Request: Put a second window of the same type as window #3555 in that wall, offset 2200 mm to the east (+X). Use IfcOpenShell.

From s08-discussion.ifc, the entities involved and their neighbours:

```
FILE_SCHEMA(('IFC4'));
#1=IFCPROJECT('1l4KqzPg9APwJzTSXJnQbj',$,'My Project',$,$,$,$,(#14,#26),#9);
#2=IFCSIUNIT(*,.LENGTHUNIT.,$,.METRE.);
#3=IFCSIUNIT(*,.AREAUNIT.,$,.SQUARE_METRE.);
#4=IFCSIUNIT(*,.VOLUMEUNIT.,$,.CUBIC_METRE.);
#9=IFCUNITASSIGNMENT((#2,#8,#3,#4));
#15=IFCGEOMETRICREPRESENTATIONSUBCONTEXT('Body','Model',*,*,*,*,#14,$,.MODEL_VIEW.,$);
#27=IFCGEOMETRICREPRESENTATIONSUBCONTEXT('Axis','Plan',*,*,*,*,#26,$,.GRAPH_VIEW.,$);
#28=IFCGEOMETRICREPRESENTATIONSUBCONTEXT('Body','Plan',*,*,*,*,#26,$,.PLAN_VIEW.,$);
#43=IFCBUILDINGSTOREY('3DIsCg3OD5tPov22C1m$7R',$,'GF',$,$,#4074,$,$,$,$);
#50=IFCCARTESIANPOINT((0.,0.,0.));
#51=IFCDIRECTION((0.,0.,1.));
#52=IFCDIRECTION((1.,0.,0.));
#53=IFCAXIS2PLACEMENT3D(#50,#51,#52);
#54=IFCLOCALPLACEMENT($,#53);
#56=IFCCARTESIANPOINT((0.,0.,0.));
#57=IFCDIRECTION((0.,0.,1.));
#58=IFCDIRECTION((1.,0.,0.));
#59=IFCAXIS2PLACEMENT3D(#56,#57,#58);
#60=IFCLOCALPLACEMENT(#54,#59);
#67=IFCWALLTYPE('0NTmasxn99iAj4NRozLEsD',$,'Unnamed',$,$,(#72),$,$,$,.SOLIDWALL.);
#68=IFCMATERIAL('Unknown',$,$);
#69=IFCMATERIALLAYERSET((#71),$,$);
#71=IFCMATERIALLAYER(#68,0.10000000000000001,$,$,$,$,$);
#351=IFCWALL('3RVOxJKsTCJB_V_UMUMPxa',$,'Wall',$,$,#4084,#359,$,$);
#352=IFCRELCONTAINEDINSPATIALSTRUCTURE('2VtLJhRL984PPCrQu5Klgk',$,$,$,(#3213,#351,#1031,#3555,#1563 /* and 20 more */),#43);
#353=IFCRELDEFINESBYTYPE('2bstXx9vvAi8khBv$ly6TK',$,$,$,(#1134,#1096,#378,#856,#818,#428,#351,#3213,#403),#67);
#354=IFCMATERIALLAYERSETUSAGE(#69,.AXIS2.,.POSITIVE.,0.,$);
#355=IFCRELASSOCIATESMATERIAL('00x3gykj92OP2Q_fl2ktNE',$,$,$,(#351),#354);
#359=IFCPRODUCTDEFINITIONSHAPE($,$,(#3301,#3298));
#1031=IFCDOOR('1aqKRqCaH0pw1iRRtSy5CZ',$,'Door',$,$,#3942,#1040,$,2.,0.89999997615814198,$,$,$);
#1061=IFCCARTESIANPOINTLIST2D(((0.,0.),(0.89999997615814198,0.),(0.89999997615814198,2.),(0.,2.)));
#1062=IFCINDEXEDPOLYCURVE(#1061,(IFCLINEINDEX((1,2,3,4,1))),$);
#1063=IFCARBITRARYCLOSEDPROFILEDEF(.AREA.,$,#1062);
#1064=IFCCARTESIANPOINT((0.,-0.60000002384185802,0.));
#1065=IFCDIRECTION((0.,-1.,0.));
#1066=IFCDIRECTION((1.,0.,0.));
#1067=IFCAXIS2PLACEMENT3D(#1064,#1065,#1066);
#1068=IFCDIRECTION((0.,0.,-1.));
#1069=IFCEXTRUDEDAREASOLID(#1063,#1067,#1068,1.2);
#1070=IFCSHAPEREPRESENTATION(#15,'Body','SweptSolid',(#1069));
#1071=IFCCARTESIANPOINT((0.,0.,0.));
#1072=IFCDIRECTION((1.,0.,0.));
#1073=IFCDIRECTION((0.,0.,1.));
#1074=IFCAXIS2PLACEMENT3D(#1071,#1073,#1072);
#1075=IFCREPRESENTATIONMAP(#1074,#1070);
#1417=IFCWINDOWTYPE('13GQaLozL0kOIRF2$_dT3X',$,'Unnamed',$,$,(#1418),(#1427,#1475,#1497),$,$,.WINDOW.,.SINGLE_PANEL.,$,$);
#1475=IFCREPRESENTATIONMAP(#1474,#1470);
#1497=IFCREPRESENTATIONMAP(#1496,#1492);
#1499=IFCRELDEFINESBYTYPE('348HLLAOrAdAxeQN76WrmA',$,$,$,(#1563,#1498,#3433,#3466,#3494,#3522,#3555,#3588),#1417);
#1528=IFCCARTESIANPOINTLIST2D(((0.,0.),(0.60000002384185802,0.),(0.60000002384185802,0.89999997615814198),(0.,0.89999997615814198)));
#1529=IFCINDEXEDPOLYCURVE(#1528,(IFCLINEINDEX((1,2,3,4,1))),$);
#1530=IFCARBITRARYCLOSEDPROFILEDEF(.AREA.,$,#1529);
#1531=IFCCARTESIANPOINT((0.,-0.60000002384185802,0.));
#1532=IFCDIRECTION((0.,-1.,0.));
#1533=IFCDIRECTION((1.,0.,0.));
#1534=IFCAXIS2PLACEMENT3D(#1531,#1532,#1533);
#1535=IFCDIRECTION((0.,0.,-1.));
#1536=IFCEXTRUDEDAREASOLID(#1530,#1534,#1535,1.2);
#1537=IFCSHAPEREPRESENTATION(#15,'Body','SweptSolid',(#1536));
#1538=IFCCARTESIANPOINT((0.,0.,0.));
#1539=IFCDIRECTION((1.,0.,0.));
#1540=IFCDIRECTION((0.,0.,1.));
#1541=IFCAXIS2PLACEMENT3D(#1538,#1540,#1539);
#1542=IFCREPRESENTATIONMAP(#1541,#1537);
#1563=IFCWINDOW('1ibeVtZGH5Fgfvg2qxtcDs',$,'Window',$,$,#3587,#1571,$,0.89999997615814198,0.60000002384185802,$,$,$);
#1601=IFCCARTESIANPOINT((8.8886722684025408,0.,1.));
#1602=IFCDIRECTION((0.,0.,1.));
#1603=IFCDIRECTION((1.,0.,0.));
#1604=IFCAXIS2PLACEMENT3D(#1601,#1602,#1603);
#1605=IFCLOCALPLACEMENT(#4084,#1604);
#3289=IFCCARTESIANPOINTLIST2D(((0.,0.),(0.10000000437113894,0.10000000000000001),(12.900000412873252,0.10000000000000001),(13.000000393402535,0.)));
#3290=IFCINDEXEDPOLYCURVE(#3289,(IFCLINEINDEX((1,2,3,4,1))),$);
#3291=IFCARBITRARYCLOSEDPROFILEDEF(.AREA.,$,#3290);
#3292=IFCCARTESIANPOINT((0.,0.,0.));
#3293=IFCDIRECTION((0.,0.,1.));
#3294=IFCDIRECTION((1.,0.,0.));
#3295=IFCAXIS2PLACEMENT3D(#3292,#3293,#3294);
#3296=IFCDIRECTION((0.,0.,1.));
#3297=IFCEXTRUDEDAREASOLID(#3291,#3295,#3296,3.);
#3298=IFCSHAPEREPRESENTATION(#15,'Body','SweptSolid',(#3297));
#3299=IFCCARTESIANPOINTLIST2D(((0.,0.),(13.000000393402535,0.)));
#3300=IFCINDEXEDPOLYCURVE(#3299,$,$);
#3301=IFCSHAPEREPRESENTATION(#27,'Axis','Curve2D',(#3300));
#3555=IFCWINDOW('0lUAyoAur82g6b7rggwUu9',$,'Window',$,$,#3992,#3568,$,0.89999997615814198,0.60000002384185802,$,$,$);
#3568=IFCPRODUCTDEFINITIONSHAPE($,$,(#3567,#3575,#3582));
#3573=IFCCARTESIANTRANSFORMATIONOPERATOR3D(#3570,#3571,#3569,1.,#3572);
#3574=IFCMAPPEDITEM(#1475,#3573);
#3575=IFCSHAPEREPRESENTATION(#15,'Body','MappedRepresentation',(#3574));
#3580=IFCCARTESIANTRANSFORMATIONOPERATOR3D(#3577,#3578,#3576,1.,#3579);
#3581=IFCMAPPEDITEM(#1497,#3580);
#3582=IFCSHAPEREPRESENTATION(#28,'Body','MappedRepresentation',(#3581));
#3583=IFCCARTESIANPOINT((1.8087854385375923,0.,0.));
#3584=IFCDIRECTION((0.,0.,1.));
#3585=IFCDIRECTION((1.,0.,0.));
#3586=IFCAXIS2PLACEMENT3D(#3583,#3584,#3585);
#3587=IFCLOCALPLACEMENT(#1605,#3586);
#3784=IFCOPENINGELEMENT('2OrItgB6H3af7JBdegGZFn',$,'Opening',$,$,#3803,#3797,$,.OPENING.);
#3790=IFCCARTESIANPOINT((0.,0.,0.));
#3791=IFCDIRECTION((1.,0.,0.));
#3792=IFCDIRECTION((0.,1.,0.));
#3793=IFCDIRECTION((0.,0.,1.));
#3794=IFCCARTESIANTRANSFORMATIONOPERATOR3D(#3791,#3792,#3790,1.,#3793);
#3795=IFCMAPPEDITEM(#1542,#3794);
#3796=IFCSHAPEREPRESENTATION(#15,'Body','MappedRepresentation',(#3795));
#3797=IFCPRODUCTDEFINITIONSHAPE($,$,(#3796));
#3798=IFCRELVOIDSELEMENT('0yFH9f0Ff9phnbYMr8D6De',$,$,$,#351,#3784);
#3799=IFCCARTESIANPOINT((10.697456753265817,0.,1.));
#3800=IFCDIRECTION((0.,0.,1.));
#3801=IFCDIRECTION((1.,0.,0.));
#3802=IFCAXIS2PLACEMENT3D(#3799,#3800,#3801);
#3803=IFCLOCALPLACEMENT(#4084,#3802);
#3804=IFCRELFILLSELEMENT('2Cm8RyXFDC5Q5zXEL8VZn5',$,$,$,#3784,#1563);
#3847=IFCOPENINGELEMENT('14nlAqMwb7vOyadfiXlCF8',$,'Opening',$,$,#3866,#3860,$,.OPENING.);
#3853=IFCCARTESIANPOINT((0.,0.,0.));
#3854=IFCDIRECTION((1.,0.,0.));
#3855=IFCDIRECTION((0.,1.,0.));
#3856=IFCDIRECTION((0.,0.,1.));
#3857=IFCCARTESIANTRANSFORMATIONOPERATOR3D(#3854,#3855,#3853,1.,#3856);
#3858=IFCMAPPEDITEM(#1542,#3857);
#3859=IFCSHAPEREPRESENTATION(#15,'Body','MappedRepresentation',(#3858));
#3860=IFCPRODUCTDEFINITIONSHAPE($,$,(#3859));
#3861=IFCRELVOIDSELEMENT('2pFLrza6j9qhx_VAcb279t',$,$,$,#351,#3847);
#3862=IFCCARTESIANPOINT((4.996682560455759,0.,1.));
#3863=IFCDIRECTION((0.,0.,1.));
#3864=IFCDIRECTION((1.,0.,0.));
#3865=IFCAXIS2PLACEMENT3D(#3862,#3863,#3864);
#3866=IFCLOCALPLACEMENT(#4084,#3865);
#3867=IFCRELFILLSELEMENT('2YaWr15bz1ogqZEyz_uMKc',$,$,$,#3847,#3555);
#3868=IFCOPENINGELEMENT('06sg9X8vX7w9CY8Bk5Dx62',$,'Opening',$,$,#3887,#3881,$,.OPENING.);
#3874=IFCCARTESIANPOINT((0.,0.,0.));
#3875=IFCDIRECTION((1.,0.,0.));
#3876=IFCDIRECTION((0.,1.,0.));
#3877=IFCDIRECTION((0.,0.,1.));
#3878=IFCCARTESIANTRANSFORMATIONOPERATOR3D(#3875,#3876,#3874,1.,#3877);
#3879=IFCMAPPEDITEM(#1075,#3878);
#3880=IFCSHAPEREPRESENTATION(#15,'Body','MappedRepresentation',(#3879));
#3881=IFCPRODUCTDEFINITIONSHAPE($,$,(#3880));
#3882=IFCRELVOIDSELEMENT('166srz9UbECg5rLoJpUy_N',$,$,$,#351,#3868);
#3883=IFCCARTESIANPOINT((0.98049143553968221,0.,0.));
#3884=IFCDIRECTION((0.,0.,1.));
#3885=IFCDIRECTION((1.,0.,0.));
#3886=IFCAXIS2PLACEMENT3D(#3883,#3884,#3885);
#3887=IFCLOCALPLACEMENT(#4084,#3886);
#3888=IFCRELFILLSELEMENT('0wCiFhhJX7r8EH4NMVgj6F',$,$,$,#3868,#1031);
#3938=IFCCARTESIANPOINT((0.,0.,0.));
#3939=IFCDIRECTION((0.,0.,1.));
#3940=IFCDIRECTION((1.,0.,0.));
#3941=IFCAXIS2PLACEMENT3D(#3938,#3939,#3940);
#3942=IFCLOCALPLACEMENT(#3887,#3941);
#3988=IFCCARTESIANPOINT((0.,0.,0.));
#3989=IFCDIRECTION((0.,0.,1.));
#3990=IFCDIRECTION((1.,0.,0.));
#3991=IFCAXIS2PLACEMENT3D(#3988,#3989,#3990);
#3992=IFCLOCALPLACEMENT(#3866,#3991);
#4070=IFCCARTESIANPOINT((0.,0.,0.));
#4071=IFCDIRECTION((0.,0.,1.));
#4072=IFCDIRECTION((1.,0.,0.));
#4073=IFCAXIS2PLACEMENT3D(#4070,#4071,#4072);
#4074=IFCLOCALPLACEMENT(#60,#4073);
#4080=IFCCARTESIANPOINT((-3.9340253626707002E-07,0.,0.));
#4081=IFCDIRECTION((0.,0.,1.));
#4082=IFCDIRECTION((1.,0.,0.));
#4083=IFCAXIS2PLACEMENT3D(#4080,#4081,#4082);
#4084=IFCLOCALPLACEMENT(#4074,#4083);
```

```python
import ifcopenshell
import ifcopenshell.api.feature
import ifcopenshell.api.geometry
import ifcopenshell.api.root
import ifcopenshell.geom
import ifcopenshell.util.element
import ifcopenshell.util.placement
import ifcopenshell.util.shape
import ifcopenshell.util.unit

model = ifcopenshell.open("s08-discussion.ifc")
unit_scale = ifcopenshell.util.unit.calculate_unit_scale(model)
settings = ifcopenshell.geom.settings()


def volume(element):
    """Net volume in cubic metres, openings subtracted."""
    shape = ifcopenshell.geom.create_shape(settings, element)
    return ifcopenshell.util.shape.get_volume(shape.geometry)


window = model.by_guid("0lUAyoAur82g6b7rggwUu9")
opening = window.FillsVoids[0].RelatingOpeningElement
wall = opening.VoidsElements[0].RelatingBuildingElement
before = volume(wall)
shift = ifcopenshell.util.placement.get_local_placement(wall.ObjectPlacement)[:3, 0] * 2.2 / unit_scale

# copy_class copies the void relationship, type, container and properties, but no geometry.
new_opening = ifcopenshell.api.root.copy_class(model, product=opening)
new_opening.Representation = ifcopenshell.util.element.copy_deep(
    model, opening.Representation, exclude=["IfcGeometricRepresentationContext", "IfcRepresentationMap"]
)
new_window = ifcopenshell.api.root.copy_class(model, product=window)
new_window.Representation = ifcopenshell.util.element.copy_deep(
    model, window.Representation, exclude=["IfcGeometricRepresentationContext", "IfcRepresentationMap"]
)
ifcopenshell.api.feature.add_filling(model, opening=new_opening, element=new_window)

for old, new in ((opening, new_opening), (window, new_window)):
    matrix = ifcopenshell.util.placement.get_local_placement(old.ObjectPlacement)
    matrix[:3, 3] += shift
    ifcopenshell.api.geometry.edit_object_placement(model, product=new, matrix=matrix, is_si=False)

after = volume(wall)

print(f"wall volume {before:.3f} -> {after:.3f} m3")

model.write("s08-discussion_updated.ifc")
```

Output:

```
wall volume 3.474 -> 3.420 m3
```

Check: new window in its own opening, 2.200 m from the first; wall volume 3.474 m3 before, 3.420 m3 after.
